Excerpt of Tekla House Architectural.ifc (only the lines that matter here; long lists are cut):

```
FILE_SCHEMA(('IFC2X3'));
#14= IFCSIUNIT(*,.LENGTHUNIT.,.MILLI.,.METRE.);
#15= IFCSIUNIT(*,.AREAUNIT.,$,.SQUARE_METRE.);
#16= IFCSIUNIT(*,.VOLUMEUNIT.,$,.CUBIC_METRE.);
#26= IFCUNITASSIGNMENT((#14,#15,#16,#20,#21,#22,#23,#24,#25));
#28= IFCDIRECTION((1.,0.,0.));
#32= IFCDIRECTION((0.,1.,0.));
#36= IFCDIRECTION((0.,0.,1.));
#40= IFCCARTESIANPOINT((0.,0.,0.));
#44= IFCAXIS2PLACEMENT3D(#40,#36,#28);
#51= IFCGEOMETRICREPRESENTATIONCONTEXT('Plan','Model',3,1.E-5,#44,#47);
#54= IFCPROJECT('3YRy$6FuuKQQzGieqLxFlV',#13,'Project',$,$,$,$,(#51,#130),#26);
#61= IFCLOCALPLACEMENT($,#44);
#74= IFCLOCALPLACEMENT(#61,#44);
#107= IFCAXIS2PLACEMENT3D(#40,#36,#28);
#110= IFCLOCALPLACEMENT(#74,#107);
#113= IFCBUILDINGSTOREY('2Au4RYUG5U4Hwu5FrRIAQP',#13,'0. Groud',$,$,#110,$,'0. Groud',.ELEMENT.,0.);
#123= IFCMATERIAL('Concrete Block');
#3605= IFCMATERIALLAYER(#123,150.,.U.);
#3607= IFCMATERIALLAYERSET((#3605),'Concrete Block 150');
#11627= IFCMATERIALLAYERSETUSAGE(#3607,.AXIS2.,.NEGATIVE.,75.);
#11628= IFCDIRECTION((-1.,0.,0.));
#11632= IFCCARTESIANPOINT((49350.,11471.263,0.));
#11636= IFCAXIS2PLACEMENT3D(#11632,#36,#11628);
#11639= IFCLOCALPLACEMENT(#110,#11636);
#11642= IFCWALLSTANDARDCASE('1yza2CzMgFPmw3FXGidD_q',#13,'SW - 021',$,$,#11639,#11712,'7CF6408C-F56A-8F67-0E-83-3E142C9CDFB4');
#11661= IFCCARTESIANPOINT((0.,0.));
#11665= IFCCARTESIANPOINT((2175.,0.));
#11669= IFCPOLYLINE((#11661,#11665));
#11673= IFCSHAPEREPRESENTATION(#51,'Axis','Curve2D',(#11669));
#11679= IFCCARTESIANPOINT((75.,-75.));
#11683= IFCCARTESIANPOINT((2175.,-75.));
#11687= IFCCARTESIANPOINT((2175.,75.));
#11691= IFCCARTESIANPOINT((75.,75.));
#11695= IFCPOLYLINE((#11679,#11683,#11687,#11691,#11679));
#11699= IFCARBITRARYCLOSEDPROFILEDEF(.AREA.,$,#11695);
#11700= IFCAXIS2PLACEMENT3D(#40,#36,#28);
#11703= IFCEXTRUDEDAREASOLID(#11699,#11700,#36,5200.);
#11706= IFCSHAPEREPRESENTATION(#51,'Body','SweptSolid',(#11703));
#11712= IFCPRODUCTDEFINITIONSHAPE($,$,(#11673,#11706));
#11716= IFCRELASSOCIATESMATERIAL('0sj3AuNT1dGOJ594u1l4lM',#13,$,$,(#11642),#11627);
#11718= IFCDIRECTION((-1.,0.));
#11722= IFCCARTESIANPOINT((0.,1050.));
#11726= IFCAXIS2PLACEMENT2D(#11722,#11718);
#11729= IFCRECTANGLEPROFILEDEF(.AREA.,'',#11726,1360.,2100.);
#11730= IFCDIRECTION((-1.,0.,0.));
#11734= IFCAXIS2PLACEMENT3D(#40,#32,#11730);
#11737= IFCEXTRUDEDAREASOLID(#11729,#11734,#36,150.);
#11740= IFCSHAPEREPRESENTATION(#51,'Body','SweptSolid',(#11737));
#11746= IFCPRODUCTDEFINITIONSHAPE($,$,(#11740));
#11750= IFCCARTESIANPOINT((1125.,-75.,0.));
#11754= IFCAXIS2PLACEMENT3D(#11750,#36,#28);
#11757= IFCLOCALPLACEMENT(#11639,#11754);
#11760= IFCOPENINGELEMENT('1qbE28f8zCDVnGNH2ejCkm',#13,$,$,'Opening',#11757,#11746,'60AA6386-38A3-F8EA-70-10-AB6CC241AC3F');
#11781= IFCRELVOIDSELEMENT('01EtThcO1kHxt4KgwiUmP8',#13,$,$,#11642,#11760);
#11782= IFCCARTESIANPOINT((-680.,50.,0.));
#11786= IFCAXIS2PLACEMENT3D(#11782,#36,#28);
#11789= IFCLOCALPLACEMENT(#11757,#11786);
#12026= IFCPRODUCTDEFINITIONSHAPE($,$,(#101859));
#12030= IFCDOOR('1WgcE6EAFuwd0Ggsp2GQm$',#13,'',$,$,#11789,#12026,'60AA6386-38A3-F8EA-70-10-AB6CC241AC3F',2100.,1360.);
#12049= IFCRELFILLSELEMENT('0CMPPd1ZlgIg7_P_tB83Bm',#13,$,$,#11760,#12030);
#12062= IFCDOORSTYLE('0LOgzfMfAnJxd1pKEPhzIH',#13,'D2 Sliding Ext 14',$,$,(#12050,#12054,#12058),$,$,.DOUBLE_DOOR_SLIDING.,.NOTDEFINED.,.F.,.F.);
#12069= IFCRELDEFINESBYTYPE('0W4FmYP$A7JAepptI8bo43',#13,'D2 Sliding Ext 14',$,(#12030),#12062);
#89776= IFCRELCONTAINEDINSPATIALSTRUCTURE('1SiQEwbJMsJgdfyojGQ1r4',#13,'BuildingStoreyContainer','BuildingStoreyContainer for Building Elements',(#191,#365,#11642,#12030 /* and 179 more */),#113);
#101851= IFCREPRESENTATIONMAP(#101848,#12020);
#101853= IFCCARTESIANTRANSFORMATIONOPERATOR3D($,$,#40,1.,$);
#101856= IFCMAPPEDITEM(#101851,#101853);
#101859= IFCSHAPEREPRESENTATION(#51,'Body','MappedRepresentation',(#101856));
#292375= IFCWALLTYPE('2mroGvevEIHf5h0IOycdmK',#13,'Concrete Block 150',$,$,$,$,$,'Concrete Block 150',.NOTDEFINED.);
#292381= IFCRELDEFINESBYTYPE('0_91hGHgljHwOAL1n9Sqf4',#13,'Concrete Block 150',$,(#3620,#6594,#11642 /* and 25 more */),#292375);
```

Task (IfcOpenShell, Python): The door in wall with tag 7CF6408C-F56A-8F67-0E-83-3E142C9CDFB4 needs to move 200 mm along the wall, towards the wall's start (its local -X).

```python
import ifcopenshell
import ifcopenshell.api.geometry
import ifcopenshell.util.placement
import ifcopenshell.util.unit

model = ifcopenshell.open("Tekla House Architectural.ifc")
unit_scale = ifcopenshell.util.unit.calculate_unit_scale(model)

door = model.by_guid("1WgcE6EAFuwd0Ggsp2GQm$")
opening = door.FillsVoids[0].RelatingOpeningElement
wall = opening.VoidsElements[0].RelatingBuildingElement

wall_matrix = ifcopenshell.util.placement.get_local_placement(wall.ObjectPlacement)
shift = wall_matrix[:3, 0] * -0.2 / unit_scale
before = ifcopenshell.util.placement.get_local_placement(door.ObjectPlacement)[:3, 3].copy()

# The door is placed relative to its opening, so it follows when the opening moves.
matrix = ifcopenshell.util.placement.get_local_placement(opening.ObjectPlacement)
matrix[:3, 3] += shift
ifcopenshell.api.geometry.edit_object_placement(
    model, product=opening, matrix=matrix, is_si=False, should_transform_children=True
)

after = ifcopenshell.util.placement.get_local_placement(door.ObjectPlacement)[:3, 3]
print("door moved by", (after - before).round(3) + 0.0)

model.write("Tekla House Architectural_updated.ifc")
```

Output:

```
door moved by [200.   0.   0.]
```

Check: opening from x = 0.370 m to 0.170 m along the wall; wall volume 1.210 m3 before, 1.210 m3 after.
